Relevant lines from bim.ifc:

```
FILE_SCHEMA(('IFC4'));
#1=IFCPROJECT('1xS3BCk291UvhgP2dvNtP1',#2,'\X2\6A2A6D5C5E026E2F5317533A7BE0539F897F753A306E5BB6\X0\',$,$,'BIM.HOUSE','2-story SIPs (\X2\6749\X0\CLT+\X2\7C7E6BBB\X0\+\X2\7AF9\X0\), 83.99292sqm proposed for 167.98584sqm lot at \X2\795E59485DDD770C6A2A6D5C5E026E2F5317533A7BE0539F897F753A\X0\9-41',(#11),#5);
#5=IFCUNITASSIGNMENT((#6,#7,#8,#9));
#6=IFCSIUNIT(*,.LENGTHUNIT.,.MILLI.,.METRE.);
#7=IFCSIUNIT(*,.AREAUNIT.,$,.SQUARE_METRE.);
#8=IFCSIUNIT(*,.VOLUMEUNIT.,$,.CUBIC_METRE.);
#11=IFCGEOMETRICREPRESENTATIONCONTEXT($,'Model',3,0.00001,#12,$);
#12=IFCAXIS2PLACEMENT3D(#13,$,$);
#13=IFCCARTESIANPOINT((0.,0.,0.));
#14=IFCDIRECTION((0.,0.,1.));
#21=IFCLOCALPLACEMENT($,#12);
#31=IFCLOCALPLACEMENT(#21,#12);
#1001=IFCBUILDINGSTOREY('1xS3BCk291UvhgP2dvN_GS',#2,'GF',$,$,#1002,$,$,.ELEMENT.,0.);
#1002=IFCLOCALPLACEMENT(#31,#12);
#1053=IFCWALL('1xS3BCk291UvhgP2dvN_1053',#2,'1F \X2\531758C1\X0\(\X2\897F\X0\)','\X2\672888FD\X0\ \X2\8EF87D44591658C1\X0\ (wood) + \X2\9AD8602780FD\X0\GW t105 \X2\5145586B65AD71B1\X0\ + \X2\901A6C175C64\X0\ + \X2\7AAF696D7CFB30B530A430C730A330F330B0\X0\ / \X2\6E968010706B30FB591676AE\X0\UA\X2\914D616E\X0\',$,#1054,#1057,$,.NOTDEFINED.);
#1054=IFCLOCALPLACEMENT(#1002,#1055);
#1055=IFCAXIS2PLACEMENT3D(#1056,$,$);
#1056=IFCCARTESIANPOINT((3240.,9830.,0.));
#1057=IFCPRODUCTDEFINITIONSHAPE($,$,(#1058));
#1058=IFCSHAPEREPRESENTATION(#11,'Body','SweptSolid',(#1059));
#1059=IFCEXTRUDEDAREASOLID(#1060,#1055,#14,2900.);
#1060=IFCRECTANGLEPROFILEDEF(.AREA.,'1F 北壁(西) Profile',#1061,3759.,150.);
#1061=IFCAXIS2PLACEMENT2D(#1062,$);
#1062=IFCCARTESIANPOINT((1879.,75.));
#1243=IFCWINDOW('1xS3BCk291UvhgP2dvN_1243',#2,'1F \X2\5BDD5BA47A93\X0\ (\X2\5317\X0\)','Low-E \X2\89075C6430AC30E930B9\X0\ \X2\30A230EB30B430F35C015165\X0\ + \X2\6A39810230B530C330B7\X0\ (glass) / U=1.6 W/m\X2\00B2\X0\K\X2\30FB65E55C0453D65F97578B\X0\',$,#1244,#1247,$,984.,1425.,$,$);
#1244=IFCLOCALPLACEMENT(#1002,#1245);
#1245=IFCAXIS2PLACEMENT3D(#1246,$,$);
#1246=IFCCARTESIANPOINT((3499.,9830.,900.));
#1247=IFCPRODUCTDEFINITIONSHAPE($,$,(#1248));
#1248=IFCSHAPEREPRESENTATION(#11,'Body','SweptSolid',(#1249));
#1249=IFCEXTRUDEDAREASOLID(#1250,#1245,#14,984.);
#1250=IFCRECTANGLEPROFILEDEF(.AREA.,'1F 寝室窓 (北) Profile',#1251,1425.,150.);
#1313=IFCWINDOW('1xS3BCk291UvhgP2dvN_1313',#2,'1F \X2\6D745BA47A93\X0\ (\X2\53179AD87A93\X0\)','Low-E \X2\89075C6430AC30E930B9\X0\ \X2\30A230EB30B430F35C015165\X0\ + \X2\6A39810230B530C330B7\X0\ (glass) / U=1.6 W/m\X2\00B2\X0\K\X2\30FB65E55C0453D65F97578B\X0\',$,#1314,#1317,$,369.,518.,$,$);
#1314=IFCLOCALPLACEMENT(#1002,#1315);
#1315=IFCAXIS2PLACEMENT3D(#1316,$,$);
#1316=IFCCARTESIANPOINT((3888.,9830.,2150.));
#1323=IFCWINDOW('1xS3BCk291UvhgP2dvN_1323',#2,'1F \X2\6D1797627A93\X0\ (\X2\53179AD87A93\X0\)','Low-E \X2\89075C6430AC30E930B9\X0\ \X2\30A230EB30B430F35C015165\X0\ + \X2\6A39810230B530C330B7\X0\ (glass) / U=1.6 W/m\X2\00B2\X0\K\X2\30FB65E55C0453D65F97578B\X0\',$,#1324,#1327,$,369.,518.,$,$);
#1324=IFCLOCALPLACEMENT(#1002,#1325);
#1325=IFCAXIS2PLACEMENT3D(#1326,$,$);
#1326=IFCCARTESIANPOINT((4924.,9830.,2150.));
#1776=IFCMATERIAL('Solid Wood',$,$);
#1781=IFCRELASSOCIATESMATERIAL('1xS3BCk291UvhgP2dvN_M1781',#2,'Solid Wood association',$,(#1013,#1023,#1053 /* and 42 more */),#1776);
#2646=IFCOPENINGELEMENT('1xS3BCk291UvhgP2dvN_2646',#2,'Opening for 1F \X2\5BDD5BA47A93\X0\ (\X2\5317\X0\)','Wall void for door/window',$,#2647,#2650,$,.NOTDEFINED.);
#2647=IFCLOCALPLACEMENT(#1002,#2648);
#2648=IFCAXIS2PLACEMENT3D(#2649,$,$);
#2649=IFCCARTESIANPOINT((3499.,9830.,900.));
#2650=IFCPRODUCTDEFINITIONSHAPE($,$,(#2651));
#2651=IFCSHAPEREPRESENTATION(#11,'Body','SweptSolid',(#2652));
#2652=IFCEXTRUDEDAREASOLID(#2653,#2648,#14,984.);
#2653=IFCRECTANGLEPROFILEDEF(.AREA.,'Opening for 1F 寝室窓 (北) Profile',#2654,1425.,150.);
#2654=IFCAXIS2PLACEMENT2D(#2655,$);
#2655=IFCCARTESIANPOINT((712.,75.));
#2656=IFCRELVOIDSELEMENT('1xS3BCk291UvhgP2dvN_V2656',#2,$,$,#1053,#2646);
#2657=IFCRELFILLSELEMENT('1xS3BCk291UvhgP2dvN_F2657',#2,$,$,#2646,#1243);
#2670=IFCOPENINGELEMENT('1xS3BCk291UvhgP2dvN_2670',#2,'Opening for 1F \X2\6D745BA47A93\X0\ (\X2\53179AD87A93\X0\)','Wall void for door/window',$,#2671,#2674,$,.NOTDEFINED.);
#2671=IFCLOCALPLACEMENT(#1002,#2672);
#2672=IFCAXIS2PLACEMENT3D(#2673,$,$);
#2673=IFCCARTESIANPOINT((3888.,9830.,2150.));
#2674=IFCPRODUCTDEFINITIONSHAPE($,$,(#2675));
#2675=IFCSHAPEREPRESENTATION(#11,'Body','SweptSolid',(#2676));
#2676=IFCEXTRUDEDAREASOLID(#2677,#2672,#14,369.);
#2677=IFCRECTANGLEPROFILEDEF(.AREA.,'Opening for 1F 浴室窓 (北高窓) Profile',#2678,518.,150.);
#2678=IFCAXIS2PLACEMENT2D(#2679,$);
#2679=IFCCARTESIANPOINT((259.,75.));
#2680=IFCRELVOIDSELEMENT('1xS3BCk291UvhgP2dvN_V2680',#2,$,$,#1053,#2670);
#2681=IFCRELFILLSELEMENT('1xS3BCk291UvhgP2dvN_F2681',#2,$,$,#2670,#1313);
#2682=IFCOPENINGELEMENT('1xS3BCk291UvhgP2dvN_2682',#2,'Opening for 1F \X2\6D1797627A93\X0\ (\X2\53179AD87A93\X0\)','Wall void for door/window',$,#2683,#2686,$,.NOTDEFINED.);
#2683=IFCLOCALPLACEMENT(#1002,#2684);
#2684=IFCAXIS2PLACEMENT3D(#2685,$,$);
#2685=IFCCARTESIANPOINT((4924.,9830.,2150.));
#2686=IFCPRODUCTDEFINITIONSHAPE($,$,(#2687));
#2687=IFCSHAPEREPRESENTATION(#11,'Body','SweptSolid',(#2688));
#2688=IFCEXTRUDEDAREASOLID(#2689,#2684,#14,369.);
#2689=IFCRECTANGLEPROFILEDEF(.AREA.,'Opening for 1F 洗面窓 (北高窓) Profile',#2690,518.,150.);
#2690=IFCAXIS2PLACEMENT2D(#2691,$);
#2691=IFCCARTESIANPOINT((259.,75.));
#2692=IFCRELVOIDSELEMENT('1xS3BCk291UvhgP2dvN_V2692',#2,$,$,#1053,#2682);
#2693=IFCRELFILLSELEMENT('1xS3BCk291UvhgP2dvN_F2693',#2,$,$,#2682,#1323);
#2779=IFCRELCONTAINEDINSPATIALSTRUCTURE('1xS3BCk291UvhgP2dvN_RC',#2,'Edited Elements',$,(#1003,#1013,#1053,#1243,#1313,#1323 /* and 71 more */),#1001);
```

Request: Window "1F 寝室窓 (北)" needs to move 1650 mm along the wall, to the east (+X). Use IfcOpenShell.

```python
import ifcopenshell
import ifcopenshell.api.geometry
import ifcopenshell.util.placement

model = ifcopenshell.open("bim.ifc")

window = model.by_guid("1xS3BCk291UvhgP2dvN_1243")
opening = window.FillsVoids[0].RelatingOpeningElement
wall = opening.VoidsElements[0].RelatingBuildingElement

wall_matrix = ifcopenshell.util.placement.get_local_placement(wall.ObjectPlacement)
shift = wall_matrix[:3, 0] * 1650.0
before = ifcopenshell.util.placement.get_local_placement(window.ObjectPlacement)[:3, 3].copy()

# The window is not placed relative to its opening, so move both.
for product in (opening, window):
    matrix = ifcopenshell.util.placement.get_local_placement(product.ObjectPlacement)
    matrix[:3, 3] += shift
    ifcopenshell.api.geometry.edit_object_placement(model, product=product, matrix=matrix, is_si=False)

after = ifcopenshell.util.placement.get_local_placement(window.ObjectPlacement)[:3, 3]
print("window moved by", (after - before).round(3) + 0.0)

model.write("bim_v2.ifc")
```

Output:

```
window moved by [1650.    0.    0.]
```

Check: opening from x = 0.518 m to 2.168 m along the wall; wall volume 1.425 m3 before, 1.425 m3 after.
